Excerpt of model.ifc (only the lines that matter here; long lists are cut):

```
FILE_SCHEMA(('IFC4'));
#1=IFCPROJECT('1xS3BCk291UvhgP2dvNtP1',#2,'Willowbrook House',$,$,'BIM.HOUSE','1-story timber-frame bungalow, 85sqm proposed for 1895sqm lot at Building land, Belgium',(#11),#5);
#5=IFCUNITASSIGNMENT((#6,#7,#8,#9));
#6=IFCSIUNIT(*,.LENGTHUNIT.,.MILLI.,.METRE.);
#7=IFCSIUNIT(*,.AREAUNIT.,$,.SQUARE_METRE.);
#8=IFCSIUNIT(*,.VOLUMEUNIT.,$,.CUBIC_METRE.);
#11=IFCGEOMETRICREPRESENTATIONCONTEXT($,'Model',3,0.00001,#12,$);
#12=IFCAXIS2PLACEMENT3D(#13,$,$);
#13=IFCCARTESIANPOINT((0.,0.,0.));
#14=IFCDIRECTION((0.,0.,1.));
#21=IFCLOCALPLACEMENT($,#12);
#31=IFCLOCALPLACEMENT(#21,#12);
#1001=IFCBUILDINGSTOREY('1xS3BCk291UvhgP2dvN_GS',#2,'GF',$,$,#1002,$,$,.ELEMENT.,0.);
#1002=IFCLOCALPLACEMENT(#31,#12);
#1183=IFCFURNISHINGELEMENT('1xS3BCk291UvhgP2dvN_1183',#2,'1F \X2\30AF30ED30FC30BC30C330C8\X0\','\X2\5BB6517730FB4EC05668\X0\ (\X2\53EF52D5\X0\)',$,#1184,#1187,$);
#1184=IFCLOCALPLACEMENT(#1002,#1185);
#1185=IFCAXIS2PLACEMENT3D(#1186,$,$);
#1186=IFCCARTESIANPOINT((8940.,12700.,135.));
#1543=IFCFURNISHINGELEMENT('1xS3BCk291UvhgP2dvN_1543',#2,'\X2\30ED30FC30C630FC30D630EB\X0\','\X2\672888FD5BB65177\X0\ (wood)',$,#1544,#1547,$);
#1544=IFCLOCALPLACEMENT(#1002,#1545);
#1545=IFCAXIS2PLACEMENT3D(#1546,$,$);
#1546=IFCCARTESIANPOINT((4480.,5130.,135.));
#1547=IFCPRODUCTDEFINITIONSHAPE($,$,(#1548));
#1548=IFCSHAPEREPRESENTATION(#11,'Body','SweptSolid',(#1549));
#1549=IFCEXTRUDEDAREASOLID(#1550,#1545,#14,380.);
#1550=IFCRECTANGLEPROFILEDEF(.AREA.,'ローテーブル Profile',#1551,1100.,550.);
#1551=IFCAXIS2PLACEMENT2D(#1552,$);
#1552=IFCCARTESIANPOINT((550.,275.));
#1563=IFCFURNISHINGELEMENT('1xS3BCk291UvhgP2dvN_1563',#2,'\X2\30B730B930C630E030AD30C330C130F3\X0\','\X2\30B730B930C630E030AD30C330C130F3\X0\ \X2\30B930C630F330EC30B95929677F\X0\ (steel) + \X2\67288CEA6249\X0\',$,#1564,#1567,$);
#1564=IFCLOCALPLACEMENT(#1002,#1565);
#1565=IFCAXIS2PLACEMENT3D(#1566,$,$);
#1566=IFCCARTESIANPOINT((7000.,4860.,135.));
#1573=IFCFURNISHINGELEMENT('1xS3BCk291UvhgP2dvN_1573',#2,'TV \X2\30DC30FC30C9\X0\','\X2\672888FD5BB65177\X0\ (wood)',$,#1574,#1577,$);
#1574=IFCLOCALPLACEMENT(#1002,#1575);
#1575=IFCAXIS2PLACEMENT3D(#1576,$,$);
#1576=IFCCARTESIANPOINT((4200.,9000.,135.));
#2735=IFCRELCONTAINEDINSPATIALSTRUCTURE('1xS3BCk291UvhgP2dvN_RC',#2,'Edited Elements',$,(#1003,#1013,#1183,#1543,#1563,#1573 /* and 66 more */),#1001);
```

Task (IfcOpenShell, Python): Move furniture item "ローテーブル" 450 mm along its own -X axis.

```python
import ifcopenshell
import ifcopenshell.api.geometry
import ifcopenshell.util.placement
import ifcopenshell.util.unit

model = ifcopenshell.open("model.ifc")
unit_scale = ifcopenshell.util.unit.calculate_unit_scale(model)

item = model.by_guid("1xS3BCk291UvhgP2dvN_1543")
matrix = ifcopenshell.util.placement.get_local_placement(item.ObjectPlacement)
matrix[:3, 3] -= matrix[:3, 0] * 0.45 / unit_scale
ifcopenshell.api.geometry.edit_object_placement(model, product=item, matrix=matrix, is_si=False)

print(ifcopenshell.util.placement.get_local_placement(item.ObjectPlacement).round(3) + 0.0)

model.write("model_updated.ifc")
```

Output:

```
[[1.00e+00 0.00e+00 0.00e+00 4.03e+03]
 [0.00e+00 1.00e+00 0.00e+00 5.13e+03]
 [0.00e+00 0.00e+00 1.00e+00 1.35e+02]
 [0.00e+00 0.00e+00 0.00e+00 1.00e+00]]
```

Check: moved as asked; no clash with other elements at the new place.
